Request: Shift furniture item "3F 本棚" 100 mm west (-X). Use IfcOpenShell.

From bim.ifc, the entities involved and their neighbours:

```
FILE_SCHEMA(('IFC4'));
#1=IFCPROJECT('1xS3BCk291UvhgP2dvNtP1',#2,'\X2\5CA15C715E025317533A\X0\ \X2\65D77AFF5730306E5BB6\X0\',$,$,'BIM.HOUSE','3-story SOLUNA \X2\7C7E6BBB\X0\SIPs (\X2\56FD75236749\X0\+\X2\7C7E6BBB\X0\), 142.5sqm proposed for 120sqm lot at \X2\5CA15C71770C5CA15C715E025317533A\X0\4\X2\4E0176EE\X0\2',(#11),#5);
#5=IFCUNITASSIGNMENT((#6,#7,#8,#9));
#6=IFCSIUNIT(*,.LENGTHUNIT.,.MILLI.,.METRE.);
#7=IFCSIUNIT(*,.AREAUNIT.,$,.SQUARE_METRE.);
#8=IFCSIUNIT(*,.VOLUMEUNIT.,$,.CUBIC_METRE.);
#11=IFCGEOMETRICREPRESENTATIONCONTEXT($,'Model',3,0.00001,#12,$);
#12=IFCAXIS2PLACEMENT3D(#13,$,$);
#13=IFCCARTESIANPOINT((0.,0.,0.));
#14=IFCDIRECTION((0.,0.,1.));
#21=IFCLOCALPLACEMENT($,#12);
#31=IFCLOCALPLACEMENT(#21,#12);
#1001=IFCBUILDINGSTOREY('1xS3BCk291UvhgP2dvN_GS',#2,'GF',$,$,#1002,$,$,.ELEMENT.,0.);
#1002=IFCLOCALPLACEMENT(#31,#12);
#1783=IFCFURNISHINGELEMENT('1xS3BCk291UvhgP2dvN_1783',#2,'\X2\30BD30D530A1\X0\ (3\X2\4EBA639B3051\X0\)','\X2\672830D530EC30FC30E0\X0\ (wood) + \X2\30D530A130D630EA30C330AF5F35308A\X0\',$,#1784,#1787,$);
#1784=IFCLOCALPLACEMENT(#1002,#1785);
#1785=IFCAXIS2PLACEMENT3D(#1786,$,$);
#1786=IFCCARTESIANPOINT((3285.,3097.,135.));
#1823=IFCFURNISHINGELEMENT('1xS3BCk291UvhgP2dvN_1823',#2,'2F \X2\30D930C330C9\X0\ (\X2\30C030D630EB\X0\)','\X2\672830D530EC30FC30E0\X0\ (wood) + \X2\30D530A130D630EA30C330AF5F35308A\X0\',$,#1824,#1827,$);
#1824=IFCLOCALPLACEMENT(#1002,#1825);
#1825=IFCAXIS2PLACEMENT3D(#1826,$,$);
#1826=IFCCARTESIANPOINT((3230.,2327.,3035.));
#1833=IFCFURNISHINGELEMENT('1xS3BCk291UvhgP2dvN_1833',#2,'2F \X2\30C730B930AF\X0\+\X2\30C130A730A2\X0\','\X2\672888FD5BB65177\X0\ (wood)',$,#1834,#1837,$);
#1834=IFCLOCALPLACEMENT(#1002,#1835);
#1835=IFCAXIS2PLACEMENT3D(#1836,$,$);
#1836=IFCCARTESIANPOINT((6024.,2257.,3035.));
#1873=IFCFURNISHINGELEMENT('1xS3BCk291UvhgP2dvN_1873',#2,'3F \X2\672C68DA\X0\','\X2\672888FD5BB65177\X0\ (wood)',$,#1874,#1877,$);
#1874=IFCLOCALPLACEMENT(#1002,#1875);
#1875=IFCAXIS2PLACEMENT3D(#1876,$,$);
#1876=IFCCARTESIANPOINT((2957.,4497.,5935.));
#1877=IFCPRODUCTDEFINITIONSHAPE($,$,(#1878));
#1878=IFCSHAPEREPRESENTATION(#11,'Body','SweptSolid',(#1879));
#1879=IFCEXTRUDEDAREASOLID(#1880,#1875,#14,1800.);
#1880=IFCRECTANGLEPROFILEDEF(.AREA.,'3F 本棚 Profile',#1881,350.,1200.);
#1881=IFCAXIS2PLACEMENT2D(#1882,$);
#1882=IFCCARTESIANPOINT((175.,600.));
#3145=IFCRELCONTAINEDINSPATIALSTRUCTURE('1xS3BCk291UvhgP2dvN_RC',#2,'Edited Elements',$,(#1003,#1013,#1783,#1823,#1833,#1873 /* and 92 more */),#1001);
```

```python
import ifcopenshell
import ifcopenshell.api.geometry
import ifcopenshell.util.placement
import ifcopenshell.util.unit

model = ifcopenshell.open("bim.ifc")
unit_scale = ifcopenshell.util.unit.calculate_unit_scale(model)

item = model.by_id(1873)
matrix = ifcopenshell.util.placement.get_local_placement(item.ObjectPlacement)
matrix[0, 3] -= 0.1 / unit_scale
ifcopenshell.api.geometry.edit_object_placement(model, product=item, matrix=matrix, is_si=False)

print(ifcopenshell.util.placement.get_local_placement(item.ObjectPlacement).round(3) + 0.0)

model.write("bim_rev.ifc")
```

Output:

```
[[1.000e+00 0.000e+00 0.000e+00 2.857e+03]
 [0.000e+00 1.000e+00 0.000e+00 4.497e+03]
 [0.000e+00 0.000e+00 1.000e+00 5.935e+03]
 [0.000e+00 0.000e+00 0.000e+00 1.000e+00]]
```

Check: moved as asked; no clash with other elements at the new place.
